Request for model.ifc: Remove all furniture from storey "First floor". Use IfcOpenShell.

First a look at what the model holds.

```python
import ifcopenshell
import ifcopenshell.util.element

model = ifcopenshell.open("model.ifc")
print(model.schema)
storey = next(s for s in model.by_type("IfcBuildingStorey") if s.Name == "First floor")
furniture = [e for e in ifcopenshell.util.element.get_decomposition(storey) if e.is_a("IfcFurnishingElement")]
seen = {}
for e in furniture:
    element_type = ifcopenshell.util.element.get_type(e)
    name = element_type.Name if element_type not in (None, e) else None
    seen[name] = seen.get(name, 0) + 1
for name, count in sorted(seen.items(), key=str):
    print(count, "x", name)
```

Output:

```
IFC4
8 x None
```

```python
import ifcopenshell
import ifcopenshell.api.root
import ifcopenshell.util.element

model = ifcopenshell.open("model.ifc")

storey = next(s for s in model.by_type("IfcBuildingStorey") if s.Name == "First floor")
furniture = [e for e in ifcopenshell.util.element.get_decomposition(storey) if e.is_a("IfcFurnishingElement")]

for e in furniture:
    ifcopenshell.api.root.remove_product(model, product=e)
print(len(furniture), "removed")

model.write("model_v2.ifc")
```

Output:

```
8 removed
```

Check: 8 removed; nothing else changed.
